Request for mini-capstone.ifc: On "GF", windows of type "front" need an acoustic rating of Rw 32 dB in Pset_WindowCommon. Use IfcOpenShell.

First a look at what the model holds.

```python
import ifcopenshell
import ifcopenshell.util.element

model = ifcopenshell.open("mini-capstone.ifc")
print(model.schema)
storey = next(s for s in model.by_type("IfcBuildingStorey") if s.Name == "GF")
windows = [e for e in ifcopenshell.util.element.get_decomposition(storey) if e.is_a("IfcWindow")]
seen = {}
for e in windows:
    element_type = ifcopenshell.util.element.get_type(e)
    key = (element_type.Name if element_type != e and element_type else None, ifcopenshell.util.element.get_pset(e, "Pset_WindowCommon", "AcousticRating"))
    seen[key] = seen.get(key, 0) + 1
for (name, value), count in sorted(seen.items(), key=str):
    print(count, "x", name, "|", value)
```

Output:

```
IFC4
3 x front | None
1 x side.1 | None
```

```python
import ifcopenshell
import ifcopenshell.api.pset
import ifcopenshell.util.element

model = ifcopenshell.open("mini-capstone.ifc")

storey = next(s for s in model.by_type("IfcBuildingStorey") if s.Name == "GF")
windows = [e for e in ifcopenshell.util.element.get_decomposition(storey) if e.is_a("IfcWindow")]

count = 0
for e in windows:
    element_type = ifcopenshell.util.element.get_type(e)
    if element_type in (None, e) or element_type.Name != "front":
        continue
    # add_pset returns the element's existing set when there is one.
    pset = ifcopenshell.api.pset.add_pset(model, product=e, name="Pset_WindowCommon")
    ifcopenshell.api.pset.edit_pset(model, pset=pset, properties={"AcousticRating": "Rw 32 dB"})
    count += 1

print(count, "windows updated")

model.write("mini-capstone_edited.ifc")
```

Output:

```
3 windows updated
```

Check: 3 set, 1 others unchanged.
